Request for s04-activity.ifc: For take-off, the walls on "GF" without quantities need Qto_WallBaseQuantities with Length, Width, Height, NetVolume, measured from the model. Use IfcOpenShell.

First a look at what the model holds.

```python
import ifcopenshell
import ifcopenshell.util.element
import ifcopenshell.util.unit

model = ifcopenshell.open("s04-activity.ifc")
print(model.schema)
for unit_type in ("LENGTHUNIT", "AREAUNIT", "VOLUMEUNIT"):
    print(unit_type, ifcopenshell.util.unit.calculate_unit_scale(model, unit_type))
storey = next(s for s in model.by_type("IfcBuildingStorey") if s.Name == "GF")
walls = [e for e in ifcopenshell.util.element.get_decomposition(storey) if e.is_a("IfcWall")]
for e in sorted(walls, key=lambda e: e.id()):
    print(e.id(), e.is_a(), e.Name, list(ifcopenshell.util.element.get_psets(e, qtos_only=True)), sep=" | ")
```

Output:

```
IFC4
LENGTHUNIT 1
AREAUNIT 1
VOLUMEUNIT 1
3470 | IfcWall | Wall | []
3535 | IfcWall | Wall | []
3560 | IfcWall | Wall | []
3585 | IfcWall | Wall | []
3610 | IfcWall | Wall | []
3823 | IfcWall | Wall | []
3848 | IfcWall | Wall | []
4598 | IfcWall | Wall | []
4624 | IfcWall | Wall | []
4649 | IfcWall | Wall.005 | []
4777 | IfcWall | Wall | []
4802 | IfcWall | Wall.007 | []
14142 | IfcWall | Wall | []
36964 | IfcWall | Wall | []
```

```python
import ifcopenshell
import ifcopenshell.api.pset
import ifcopenshell.geom
import ifcopenshell.util.element
import ifcopenshell.util.shape
import ifcopenshell.util.unit

model = ifcopenshell.open("s04-activity.ifc")
unit_scale = ifcopenshell.util.unit.calculate_unit_scale(model)
volume_scale = ifcopenshell.util.unit.calculate_unit_scale(model, "VOLUMEUNIT")
settings = ifcopenshell.geom.settings()

storey = next(s for s in model.by_type("IfcBuildingStorey") if s.Name == "GF")
walls = [e for e in ifcopenshell.util.element.get_decomposition(storey) if e.is_a("IfcWall")]

for e in sorted(walls, key=lambda e: e.id()):
    if ifcopenshell.util.element.get_psets(e, qtos_only=True, should_inherit=False):
        continue
    # Geometry comes back in metres, in the element's own axes.
    shape = ifcopenshell.geom.create_shape(settings, e)
    values = {
        "Length": ifcopenshell.util.shape.get_x(shape.geometry) / unit_scale,
        "Width": ifcopenshell.util.shape.get_y(shape.geometry) / unit_scale,
        "Height": ifcopenshell.util.shape.get_z(shape.geometry) / unit_scale,
        "NetVolume": ifcopenshell.util.shape.get_volume(shape.geometry) / volume_scale,
    }
    qto = ifcopenshell.api.pset.add_qto(model, product=e, name="Qto_WallBaseQuantities")
    ifcopenshell.api.pset.edit_qto(model, qto=qto, properties=values)
    print(e.id(), {k: round(v, 3) for k, v in values.items()})

model.write("s04-activity_rev.ifc")
```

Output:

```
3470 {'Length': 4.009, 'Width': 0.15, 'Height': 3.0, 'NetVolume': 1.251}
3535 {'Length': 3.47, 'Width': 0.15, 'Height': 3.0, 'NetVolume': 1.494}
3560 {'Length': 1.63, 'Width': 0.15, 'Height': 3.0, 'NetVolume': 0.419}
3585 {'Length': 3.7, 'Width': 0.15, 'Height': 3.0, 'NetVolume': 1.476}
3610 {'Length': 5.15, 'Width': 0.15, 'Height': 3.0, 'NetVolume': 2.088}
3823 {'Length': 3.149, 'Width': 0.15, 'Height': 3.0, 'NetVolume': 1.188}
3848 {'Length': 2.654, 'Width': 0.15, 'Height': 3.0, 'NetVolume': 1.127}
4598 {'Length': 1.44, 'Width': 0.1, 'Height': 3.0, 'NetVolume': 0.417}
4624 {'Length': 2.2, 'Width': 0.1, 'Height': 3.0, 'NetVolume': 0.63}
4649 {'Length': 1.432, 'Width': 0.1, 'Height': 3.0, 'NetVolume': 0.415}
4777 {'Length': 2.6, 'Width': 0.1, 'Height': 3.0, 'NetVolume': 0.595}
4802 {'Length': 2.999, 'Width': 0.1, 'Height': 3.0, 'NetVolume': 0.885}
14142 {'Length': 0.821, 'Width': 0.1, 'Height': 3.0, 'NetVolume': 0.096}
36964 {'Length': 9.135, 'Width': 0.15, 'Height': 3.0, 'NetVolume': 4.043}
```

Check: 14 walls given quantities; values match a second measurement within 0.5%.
